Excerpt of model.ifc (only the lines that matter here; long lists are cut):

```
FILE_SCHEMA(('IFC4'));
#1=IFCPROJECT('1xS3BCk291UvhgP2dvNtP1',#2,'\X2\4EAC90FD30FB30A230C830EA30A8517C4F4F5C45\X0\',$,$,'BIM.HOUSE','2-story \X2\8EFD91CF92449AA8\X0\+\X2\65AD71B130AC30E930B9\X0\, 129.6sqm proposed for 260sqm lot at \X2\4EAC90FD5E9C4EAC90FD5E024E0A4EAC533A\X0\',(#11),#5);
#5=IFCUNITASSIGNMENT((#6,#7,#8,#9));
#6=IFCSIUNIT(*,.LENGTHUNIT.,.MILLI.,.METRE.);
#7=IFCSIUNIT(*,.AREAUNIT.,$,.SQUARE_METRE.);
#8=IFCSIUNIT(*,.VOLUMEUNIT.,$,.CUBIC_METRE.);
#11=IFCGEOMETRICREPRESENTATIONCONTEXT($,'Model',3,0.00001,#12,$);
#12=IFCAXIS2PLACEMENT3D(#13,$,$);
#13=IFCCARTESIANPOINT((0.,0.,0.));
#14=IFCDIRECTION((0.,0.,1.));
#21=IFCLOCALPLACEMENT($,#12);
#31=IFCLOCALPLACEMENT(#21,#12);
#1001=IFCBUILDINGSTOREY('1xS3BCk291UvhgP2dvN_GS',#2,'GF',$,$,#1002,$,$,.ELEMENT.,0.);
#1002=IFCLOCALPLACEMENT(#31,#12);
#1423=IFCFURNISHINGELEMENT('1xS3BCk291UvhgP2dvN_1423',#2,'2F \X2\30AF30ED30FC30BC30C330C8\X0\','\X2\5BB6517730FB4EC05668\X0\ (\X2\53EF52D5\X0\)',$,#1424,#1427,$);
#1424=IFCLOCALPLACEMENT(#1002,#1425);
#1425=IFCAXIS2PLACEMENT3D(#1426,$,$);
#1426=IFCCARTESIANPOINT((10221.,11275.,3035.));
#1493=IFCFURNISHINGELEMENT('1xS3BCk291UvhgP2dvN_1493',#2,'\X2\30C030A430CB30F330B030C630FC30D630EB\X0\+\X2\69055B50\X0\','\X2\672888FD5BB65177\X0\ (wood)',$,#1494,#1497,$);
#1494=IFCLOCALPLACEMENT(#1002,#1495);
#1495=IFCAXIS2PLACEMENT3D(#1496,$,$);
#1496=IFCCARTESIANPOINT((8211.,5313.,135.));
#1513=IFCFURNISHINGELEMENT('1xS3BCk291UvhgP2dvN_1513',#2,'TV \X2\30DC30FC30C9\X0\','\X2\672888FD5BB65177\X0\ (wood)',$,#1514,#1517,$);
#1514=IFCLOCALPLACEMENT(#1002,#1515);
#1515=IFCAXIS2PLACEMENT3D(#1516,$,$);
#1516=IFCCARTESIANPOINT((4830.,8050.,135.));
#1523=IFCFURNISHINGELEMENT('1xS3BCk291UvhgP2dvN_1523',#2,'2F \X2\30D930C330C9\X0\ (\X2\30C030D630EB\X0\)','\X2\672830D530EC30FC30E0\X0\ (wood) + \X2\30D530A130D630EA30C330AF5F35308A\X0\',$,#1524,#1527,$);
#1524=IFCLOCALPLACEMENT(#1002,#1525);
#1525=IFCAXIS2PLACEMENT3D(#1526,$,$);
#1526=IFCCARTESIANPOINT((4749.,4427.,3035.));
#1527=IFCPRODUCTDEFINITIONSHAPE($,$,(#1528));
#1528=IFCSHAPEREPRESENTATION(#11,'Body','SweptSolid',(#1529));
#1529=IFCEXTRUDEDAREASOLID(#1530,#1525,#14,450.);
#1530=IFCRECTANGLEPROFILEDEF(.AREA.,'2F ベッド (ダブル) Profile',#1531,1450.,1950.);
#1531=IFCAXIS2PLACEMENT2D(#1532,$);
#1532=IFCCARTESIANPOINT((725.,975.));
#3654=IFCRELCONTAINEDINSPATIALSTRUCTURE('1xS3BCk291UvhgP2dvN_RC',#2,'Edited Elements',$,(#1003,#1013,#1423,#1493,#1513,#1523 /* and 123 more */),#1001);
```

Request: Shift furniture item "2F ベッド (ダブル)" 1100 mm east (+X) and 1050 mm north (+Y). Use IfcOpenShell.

```python
import ifcopenshell
import ifcopenshell.api.geometry
import ifcopenshell.util.placement

model = ifcopenshell.open("model.ifc")

item = model.by_guid("1xS3BCk291UvhgP2dvN_1523")
matrix = ifcopenshell.util.placement.get_local_placement(item.ObjectPlacement)
matrix[0, 3] += 1100.0
matrix[1, 3] += 1050.0
ifcopenshell.api.geometry.edit_object_placement(model, product=item, matrix=matrix, is_si=False)

print(ifcopenshell.util.placement.get_local_placement(item.ObjectPlacement).round(3) + 0.0)

model.write("model_v2.ifc")
```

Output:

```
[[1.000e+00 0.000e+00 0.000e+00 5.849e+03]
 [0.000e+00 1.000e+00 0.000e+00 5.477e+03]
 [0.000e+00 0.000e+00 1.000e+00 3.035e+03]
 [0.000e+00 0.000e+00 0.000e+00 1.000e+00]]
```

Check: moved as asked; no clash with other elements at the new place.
